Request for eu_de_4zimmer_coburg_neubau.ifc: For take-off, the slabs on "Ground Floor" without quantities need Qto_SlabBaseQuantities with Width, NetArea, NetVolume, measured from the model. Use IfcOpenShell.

First a look at what the model holds.

```python
import ifcopenshell
import ifcopenshell.util.element
import ifcopenshell.util.unit

model = ifcopenshell.open("eu_de_4zimmer_coburg_neubau.ifc")
print(model.schema)
for unit_type in ("LENGTHUNIT", "AREAUNIT", "VOLUMEUNIT"):
    print(unit_type, ifcopenshell.util.unit.calculate_unit_scale(model, unit_type))
storey = next(s for s in model.by_type("IfcBuildingStorey") if s.Name == "Ground Floor")
slabs = [e for e in ifcopenshell.util.element.get_decomposition(storey) if e.is_a("IfcSlab")]
for e in sorted(slabs, key=lambda e: e.id()):
    print(e.id(), e.is_a(), e.Name, list(ifcopenshell.util.element.get_psets(e, qtos_only=True)), sep=" | ")
```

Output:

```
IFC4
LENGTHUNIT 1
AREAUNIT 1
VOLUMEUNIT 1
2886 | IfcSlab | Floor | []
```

```python
import ifcopenshell
import ifcopenshell.api.pset
import ifcopenshell.geom
import ifcopenshell.util.element
import ifcopenshell.util.shape
import ifcopenshell.util.unit

model = ifcopenshell.open("eu_de_4zimmer_coburg_neubau.ifc")
unit_scale = ifcopenshell.util.unit.calculate_unit_scale(model)
area_scale = ifcopenshell.util.unit.calculate_unit_scale(model, "AREAUNIT")
volume_scale = ifcopenshell.util.unit.calculate_unit_scale(model, "VOLUMEUNIT")
settings = ifcopenshell.geom.settings()

storey = next(s for s in model.by_type("IfcBuildingStorey") if s.Name == "Ground Floor")
slabs = [e for e in ifcopenshell.util.element.get_decomposition(storey) if e.is_a("IfcSlab")]

for e in sorted(slabs, key=lambda e: e.id()):
    if ifcopenshell.util.element.get_psets(e, qtos_only=True, should_inherit=False):
        continue
    # Geometry comes back in metres, in the element's own axes.
    shape = ifcopenshell.geom.create_shape(settings, e)
    values = {
        "Width": ifcopenshell.util.shape.get_z(shape.geometry) / unit_scale,
        "NetArea": ifcopenshell.util.shape.get_footprint_area(shape.geometry) / area_scale,
        "NetVolume": ifcopenshell.util.shape.get_volume(shape.geometry) / volume_scale,
    }
    qto = ifcopenshell.api.pset.add_qto(model, product=e, name="Qto_SlabBaseQuantities")
    ifcopenshell.api.pset.edit_qto(model, qto=qto, properties=values)
    print(e.id(), {k: round(v, 3) for k, v in values.items()})

model.write("eu_de_4zimmer_coburg_neubau_updated.ifc")
```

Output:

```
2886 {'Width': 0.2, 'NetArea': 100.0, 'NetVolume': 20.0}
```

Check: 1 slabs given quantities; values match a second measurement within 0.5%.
